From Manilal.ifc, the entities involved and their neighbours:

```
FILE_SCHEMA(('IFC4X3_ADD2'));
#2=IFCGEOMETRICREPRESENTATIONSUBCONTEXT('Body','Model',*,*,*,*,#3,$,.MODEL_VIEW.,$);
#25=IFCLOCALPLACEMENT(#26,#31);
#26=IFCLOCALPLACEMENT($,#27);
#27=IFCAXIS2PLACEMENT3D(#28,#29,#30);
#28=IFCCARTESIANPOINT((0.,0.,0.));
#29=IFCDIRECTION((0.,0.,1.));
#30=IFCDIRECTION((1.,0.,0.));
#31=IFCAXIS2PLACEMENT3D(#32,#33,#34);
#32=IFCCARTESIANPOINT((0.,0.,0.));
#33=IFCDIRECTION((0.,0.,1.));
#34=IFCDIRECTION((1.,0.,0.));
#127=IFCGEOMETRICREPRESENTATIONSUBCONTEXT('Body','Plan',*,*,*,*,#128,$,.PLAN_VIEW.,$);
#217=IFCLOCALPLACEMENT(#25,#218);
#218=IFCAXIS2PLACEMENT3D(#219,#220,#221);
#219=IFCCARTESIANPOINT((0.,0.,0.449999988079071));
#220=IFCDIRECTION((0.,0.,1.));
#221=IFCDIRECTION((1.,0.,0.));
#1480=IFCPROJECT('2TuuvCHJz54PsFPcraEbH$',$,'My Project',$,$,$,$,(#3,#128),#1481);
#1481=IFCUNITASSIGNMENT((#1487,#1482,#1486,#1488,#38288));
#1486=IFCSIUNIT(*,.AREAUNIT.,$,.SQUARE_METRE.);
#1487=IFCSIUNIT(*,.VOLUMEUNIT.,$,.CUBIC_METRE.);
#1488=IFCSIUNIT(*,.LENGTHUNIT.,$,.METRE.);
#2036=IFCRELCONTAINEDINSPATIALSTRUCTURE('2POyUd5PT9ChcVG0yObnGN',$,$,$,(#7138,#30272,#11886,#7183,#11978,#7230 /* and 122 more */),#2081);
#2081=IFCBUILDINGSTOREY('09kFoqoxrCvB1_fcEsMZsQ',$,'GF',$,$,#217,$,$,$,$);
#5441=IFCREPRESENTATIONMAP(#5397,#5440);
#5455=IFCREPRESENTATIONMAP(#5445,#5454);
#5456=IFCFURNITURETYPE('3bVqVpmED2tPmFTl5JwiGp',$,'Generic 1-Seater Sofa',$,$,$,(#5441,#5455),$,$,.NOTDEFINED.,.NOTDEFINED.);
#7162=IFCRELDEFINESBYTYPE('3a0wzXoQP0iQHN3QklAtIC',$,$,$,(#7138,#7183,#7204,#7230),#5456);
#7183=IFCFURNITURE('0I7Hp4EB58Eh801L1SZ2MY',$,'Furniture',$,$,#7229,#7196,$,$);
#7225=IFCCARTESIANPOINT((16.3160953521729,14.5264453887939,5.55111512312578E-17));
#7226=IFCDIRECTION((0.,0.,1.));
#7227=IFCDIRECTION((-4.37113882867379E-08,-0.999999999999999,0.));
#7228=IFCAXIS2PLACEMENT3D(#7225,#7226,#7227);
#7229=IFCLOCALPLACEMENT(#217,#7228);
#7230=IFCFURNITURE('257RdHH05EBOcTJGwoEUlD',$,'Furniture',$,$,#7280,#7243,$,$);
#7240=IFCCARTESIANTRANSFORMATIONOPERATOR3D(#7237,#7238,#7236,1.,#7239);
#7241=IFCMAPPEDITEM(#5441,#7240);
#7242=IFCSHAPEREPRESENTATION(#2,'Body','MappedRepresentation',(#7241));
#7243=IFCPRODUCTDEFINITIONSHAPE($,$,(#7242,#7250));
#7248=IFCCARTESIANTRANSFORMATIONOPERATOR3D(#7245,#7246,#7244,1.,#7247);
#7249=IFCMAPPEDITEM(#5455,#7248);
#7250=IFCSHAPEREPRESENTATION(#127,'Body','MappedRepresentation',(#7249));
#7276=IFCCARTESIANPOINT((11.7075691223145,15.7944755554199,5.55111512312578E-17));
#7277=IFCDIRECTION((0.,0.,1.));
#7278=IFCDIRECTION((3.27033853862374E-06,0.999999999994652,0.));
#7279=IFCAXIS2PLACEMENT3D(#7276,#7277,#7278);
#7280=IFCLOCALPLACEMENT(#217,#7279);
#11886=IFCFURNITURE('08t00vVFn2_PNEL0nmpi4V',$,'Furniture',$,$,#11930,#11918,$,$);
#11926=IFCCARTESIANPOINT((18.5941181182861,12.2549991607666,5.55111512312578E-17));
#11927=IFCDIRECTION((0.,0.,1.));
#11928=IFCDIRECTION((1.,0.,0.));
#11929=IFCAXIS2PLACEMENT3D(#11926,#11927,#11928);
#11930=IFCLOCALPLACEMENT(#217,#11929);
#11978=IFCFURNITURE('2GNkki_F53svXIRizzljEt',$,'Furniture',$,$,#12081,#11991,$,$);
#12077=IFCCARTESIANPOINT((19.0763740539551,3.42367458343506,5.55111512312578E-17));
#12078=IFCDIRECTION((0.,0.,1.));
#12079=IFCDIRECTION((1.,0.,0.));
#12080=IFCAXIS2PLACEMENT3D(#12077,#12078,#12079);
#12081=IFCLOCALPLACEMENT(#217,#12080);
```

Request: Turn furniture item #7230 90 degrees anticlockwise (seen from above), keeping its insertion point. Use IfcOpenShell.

```python
import ifcopenshell
import ifcopenshell.api.geometry
import ifcopenshell.util.placement

model = ifcopenshell.open("Manilal.ifc")

item = model.by_guid("257RdHH05EBOcTJGwoEUlD")
matrix = ifcopenshell.util.placement.get_local_placement(item.ObjectPlacement)
matrix = matrix @ ifcopenshell.util.placement.rotation(90, "Z")
ifcopenshell.api.geometry.edit_object_placement(model, product=item, matrix=matrix, is_si=False)

print(ifcopenshell.util.placement.get_local_placement(item.ObjectPlacement).round(3) + 0.0)

model.write("Manilal-out.ifc")
```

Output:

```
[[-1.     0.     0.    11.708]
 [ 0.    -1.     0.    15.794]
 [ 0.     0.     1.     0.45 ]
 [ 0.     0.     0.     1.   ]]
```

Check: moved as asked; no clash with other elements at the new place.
